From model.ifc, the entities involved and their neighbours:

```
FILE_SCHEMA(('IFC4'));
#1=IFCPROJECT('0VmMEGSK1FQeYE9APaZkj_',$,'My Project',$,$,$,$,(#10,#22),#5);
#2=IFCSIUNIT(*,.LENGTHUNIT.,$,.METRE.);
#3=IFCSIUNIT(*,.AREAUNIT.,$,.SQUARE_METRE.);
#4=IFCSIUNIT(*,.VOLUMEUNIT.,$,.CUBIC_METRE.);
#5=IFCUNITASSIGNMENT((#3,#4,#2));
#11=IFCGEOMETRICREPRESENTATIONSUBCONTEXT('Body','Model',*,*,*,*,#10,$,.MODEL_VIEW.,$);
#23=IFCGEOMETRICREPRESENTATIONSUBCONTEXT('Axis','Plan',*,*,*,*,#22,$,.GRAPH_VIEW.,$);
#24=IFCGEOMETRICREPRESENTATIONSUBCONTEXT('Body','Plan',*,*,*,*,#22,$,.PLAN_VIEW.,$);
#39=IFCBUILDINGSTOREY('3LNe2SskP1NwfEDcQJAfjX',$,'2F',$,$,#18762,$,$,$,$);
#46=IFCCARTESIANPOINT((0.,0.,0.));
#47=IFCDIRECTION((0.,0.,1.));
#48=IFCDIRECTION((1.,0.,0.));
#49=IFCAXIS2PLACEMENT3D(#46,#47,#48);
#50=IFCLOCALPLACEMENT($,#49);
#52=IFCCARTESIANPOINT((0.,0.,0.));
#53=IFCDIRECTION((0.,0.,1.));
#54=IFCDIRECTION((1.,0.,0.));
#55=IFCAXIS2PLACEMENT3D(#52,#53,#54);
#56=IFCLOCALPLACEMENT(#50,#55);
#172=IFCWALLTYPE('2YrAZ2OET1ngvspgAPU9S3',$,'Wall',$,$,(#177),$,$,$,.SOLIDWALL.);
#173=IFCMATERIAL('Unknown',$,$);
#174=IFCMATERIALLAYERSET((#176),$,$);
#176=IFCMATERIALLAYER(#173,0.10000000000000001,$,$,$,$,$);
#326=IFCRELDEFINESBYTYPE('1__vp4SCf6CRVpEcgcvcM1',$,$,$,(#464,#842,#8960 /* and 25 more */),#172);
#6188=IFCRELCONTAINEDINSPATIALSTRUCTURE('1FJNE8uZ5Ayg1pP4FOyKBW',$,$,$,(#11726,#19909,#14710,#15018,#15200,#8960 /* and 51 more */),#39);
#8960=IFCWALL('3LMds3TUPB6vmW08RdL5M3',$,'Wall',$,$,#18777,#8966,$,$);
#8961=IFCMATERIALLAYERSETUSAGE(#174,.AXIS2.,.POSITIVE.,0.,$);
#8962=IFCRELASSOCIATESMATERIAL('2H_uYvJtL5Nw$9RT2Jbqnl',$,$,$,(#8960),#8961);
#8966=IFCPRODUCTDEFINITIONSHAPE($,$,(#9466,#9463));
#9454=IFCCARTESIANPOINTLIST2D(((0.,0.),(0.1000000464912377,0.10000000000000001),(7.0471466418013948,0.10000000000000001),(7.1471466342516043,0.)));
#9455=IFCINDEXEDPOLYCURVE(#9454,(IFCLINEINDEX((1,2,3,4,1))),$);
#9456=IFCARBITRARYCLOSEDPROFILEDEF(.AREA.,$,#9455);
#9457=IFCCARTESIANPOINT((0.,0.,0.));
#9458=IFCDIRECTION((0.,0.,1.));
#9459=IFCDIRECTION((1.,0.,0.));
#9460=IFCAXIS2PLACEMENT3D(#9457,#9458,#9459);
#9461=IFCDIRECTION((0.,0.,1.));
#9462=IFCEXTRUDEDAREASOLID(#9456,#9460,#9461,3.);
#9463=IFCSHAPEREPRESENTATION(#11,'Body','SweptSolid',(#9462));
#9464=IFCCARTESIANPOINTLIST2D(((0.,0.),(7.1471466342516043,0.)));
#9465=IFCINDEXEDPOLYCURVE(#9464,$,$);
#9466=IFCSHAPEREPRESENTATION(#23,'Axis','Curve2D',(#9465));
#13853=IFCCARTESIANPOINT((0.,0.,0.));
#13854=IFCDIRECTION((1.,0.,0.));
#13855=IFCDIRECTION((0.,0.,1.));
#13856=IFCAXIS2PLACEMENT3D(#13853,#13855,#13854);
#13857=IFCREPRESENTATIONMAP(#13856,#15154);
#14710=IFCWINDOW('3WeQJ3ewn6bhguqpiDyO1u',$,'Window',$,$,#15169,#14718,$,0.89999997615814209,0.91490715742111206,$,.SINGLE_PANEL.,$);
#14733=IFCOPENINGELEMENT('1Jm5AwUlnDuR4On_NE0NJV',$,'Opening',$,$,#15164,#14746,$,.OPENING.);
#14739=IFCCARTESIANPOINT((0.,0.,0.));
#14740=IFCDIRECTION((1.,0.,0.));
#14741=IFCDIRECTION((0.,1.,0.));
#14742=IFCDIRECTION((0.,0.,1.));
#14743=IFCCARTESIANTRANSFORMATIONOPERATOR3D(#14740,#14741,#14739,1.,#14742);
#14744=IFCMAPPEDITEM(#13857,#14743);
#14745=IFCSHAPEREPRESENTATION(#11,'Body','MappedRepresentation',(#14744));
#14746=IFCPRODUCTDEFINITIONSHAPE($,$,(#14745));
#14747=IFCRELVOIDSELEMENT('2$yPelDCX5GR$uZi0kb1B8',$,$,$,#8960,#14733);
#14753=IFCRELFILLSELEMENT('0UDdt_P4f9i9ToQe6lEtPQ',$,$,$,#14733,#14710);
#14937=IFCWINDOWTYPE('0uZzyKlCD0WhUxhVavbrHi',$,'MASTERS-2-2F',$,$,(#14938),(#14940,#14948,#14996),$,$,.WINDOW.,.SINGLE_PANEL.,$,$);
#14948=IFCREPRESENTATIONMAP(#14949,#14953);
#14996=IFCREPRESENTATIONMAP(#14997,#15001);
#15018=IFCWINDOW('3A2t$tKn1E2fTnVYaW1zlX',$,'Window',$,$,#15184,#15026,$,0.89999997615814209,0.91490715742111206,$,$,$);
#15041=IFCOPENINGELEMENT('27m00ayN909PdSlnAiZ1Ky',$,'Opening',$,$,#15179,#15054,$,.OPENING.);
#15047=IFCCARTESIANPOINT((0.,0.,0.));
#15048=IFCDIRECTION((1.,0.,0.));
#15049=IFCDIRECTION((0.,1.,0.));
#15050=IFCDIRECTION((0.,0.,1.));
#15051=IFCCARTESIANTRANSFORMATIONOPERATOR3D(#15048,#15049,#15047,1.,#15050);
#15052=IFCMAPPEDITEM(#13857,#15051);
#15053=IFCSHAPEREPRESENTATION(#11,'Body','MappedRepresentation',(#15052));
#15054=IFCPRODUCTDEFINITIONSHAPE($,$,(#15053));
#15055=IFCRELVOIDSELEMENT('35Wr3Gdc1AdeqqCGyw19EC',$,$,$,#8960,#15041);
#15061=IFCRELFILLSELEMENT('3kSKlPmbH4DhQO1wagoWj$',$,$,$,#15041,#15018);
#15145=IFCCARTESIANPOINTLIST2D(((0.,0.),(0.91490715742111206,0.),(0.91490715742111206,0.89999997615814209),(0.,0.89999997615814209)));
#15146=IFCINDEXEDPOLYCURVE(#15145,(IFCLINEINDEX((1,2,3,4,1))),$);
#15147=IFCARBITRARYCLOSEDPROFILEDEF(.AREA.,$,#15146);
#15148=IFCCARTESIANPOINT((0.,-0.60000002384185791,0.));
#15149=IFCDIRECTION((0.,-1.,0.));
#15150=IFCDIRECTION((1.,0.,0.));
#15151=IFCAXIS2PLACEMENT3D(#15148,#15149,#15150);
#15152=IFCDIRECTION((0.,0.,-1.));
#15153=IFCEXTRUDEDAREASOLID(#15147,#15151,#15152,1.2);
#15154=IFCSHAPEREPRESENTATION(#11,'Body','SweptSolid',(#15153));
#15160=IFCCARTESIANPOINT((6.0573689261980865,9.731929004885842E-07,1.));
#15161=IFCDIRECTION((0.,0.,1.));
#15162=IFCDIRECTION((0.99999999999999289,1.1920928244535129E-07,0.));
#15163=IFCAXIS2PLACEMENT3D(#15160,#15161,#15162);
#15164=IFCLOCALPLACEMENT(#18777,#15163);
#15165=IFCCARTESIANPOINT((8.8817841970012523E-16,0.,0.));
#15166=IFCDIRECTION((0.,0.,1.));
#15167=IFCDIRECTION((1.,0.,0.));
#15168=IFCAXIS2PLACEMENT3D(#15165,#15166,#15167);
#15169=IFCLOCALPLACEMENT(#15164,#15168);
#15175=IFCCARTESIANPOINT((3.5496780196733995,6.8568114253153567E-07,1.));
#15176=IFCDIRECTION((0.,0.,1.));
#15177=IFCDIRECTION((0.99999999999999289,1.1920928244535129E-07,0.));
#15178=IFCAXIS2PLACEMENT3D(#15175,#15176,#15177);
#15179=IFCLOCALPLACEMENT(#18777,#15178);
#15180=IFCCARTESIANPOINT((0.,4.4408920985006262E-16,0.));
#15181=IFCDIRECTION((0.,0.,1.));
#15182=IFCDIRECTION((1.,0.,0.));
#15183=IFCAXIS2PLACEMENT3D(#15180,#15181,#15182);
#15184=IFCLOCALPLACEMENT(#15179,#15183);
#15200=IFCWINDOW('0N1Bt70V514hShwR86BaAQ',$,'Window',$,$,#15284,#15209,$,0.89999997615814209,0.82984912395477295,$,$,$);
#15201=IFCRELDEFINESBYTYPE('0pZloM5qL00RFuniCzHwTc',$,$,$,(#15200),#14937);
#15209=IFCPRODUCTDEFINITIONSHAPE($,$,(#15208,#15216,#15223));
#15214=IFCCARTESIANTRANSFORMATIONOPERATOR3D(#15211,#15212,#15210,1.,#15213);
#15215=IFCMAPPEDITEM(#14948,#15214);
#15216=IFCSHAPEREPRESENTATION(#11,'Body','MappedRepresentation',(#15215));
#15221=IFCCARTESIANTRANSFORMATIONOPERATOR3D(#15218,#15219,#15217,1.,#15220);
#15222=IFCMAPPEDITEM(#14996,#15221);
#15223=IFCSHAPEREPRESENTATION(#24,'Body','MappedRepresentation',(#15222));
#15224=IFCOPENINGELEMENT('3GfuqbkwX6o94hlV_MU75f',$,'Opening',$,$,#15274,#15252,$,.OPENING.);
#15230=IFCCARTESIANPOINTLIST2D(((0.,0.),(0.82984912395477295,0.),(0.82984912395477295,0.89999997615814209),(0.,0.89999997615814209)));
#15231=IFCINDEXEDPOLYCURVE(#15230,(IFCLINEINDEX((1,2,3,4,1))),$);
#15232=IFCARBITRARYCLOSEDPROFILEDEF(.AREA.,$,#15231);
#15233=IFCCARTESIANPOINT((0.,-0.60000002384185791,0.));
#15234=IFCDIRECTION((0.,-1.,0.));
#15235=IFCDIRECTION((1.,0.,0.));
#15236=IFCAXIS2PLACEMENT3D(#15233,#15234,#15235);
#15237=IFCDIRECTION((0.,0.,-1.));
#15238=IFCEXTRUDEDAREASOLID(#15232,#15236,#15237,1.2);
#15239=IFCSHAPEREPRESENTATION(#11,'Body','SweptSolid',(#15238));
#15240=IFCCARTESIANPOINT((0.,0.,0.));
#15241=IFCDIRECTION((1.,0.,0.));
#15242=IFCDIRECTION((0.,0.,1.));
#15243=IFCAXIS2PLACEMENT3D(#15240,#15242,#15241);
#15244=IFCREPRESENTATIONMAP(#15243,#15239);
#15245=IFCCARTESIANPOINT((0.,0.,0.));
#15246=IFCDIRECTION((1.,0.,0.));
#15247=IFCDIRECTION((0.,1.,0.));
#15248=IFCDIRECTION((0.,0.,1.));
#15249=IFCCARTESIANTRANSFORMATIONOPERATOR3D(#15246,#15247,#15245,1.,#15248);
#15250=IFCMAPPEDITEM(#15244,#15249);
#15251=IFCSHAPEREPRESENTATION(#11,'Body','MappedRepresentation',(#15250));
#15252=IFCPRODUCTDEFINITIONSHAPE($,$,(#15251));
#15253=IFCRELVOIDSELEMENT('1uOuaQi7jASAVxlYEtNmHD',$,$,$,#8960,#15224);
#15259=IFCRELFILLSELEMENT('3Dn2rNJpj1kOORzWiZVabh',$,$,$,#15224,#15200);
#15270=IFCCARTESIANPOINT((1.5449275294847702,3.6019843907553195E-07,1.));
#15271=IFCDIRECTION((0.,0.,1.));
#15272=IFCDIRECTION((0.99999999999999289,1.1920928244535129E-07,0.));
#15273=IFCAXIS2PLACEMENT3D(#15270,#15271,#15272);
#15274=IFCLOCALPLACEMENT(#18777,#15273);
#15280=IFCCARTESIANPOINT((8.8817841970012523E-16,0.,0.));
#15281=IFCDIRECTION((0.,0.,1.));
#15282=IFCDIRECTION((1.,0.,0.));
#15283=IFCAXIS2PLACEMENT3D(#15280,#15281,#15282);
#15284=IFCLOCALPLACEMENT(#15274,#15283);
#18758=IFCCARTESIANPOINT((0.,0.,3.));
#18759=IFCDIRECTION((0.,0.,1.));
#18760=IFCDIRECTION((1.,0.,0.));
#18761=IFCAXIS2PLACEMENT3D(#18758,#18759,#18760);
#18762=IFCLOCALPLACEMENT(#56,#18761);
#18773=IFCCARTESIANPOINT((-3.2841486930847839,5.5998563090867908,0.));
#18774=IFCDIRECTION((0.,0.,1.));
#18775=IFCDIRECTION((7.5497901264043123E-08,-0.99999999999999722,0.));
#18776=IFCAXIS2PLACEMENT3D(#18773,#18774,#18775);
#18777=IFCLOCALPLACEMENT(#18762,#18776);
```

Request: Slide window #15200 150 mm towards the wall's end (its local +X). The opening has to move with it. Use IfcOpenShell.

```python
import ifcopenshell
import ifcopenshell.api.geometry
import ifcopenshell.util.placement

model = ifcopenshell.open("model.ifc")

window = model.by_guid("0N1Bt70V514hShwR86BaAQ")
opening = window.FillsVoids[0].RelatingOpeningElement
wall = opening.VoidsElements[0].RelatingBuildingElement

wall_matrix = ifcopenshell.util.placement.get_local_placement(wall.ObjectPlacement)
shift = wall_matrix[:3, 0] * 0.15
before = ifcopenshell.util.placement.get_local_placement(window.ObjectPlacement)[:3, 3].copy()

# The window is placed relative to its opening, so it follows when the opening moves.
matrix = ifcopenshell.util.placement.get_local_placement(opening.ObjectPlacement)
matrix[:3, 3] += shift
ifcopenshell.api.geometry.edit_object_placement(
    model, product=opening, matrix=matrix, is_si=False, should_transform_children=True
)

after = ifcopenshell.util.placement.get_local_placement(window.ObjectPlacement)[:3, 3]
print("window moved by", (after - before).round(3) + 0.0)

model.write("model_rev.ifc")
```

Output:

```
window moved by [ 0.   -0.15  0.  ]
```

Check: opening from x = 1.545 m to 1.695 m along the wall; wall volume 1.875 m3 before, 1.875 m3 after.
